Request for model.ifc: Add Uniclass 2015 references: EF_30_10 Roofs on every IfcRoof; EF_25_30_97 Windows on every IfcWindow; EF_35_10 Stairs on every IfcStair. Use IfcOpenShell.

First a look at what the model holds.

```python
import ifcopenshell

model = ifcopenshell.open("model.ifc")
print(model.schema)
print("classifications:", [c.Name for c in model.by_type("IfcClassification")])
for ifc_class in ("IfcDoor", "IfcRoof", "IfcStair", "IfcWall", "IfcWindow"):
    print(ifc_class, len(model.by_type(ifc_class)))
```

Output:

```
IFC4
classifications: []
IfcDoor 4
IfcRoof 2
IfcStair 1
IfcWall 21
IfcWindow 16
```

```python
import ifcopenshell
import ifcopenshell.api.classification

model = ifcopenshell.open("model.ifc")

system = ifcopenshell.api.classification.add_classification(model, classification="Uniclass 2015")

codes = {
    "IfcRoof": ("EF_30_10", "Roofs"),
    "IfcWindow": ("EF_25_30_97", "Windows"),
    "IfcStair": ("EF_35_10", "Stairs"),
}
for ifc_class, (code, name) in codes.items():
    products = model.by_type(ifc_class)
    ifcopenshell.api.classification.add_reference(
        model, products=products, classification=system, identification=code, name=name
    )
    print(code, len(products))

model.write("model_updated.ifc")
```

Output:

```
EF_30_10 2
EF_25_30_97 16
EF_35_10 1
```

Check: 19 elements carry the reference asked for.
